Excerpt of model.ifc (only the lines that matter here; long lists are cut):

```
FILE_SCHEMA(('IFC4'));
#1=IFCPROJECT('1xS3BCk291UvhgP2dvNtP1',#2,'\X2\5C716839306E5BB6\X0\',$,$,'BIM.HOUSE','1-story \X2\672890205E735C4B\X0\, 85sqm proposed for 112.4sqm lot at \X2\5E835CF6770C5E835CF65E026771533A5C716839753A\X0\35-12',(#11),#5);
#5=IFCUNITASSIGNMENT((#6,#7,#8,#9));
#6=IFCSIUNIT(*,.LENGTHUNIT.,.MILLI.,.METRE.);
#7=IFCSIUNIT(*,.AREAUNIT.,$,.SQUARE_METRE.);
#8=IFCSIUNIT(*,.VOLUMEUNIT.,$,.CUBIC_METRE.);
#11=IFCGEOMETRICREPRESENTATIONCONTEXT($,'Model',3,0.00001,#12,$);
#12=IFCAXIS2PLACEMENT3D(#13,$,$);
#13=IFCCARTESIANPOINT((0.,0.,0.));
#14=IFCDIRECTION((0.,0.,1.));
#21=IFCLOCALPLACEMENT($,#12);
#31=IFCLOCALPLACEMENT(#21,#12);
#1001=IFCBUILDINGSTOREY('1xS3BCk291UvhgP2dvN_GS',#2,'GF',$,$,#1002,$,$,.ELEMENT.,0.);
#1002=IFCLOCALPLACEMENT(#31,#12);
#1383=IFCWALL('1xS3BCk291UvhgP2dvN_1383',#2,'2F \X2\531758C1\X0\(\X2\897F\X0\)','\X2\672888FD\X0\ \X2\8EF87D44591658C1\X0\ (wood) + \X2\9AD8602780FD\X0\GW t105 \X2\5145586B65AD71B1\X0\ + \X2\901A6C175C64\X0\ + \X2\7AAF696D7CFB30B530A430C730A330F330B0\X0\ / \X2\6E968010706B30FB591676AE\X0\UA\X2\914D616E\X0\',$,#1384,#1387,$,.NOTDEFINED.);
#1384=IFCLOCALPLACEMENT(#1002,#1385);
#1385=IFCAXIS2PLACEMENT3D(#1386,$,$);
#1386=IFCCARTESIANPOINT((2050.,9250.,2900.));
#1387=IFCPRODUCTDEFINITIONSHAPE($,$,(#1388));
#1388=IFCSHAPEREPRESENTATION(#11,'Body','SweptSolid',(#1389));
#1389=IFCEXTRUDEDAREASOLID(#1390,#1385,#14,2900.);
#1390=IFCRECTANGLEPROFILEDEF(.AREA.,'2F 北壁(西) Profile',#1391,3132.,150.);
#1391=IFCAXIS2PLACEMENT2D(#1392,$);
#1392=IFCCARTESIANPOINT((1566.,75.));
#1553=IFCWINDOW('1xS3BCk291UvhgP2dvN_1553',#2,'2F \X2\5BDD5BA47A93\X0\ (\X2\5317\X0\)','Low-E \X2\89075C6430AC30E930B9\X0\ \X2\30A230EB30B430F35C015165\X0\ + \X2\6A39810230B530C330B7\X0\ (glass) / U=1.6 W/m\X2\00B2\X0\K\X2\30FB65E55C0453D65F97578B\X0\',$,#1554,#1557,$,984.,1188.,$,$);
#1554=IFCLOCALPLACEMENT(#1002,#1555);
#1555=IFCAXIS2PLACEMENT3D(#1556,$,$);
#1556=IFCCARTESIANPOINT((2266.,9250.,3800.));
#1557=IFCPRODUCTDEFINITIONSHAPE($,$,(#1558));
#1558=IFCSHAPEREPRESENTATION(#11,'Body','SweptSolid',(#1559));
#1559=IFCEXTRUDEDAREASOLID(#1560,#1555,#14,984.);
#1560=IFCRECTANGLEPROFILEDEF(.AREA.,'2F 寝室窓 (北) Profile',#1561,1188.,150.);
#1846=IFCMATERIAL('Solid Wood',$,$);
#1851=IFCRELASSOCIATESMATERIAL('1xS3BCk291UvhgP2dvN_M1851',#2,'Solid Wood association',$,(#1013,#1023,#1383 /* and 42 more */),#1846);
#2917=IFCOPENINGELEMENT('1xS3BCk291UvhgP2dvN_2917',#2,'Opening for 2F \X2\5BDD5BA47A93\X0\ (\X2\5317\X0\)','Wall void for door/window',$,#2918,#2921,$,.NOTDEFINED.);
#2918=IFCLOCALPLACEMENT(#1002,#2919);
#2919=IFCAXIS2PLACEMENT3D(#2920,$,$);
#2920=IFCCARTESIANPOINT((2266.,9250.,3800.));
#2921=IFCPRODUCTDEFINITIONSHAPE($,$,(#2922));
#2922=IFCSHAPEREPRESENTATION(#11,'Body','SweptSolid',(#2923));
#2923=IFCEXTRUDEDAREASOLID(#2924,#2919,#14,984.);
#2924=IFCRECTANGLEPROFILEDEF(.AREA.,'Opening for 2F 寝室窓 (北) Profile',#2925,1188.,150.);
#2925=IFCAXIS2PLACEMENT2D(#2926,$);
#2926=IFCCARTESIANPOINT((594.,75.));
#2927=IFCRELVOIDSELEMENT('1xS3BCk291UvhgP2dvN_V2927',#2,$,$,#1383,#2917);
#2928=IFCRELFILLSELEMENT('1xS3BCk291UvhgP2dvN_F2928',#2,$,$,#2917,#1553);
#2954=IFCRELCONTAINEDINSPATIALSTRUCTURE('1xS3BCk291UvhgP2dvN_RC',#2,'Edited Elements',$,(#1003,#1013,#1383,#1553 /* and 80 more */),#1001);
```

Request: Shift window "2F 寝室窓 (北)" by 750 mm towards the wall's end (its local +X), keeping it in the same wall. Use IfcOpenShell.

```python
import ifcopenshell
import ifcopenshell.api.geometry
import ifcopenshell.util.placement
import ifcopenshell.util.unit

model = ifcopenshell.open("model.ifc")
unit_scale = ifcopenshell.util.unit.calculate_unit_scale(model)

window = model.by_guid("1xS3BCk291UvhgP2dvN_1553")
opening = window.FillsVoids[0].RelatingOpeningElement
wall = opening.VoidsElements[0].RelatingBuildingElement

wall_matrix = ifcopenshell.util.placement.get_local_placement(wall.ObjectPlacement)
shift = wall_matrix[:3, 0] * 0.75 / unit_scale
before = ifcopenshell.util.placement.get_local_placement(window.ObjectPlacement)[:3, 3].copy()

# The window is not placed relative to its opening, so move both.
for product in (opening, window):
    matrix = ifcopenshell.util.placement.get_local_placement(product.ObjectPlacement)
    matrix[:3, 3] += shift
    ifcopenshell.api.geometry.edit_object_placement(model, product=product, matrix=matrix, is_si=False)

after = ifcopenshell.util.placement.get_local_placement(window.ObjectPlacement)[:3, 3]
print("window moved by", (after - before).round(3) + 0.0)

model.write("model_edited.ifc")
```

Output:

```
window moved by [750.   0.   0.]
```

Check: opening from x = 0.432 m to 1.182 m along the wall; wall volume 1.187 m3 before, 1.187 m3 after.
